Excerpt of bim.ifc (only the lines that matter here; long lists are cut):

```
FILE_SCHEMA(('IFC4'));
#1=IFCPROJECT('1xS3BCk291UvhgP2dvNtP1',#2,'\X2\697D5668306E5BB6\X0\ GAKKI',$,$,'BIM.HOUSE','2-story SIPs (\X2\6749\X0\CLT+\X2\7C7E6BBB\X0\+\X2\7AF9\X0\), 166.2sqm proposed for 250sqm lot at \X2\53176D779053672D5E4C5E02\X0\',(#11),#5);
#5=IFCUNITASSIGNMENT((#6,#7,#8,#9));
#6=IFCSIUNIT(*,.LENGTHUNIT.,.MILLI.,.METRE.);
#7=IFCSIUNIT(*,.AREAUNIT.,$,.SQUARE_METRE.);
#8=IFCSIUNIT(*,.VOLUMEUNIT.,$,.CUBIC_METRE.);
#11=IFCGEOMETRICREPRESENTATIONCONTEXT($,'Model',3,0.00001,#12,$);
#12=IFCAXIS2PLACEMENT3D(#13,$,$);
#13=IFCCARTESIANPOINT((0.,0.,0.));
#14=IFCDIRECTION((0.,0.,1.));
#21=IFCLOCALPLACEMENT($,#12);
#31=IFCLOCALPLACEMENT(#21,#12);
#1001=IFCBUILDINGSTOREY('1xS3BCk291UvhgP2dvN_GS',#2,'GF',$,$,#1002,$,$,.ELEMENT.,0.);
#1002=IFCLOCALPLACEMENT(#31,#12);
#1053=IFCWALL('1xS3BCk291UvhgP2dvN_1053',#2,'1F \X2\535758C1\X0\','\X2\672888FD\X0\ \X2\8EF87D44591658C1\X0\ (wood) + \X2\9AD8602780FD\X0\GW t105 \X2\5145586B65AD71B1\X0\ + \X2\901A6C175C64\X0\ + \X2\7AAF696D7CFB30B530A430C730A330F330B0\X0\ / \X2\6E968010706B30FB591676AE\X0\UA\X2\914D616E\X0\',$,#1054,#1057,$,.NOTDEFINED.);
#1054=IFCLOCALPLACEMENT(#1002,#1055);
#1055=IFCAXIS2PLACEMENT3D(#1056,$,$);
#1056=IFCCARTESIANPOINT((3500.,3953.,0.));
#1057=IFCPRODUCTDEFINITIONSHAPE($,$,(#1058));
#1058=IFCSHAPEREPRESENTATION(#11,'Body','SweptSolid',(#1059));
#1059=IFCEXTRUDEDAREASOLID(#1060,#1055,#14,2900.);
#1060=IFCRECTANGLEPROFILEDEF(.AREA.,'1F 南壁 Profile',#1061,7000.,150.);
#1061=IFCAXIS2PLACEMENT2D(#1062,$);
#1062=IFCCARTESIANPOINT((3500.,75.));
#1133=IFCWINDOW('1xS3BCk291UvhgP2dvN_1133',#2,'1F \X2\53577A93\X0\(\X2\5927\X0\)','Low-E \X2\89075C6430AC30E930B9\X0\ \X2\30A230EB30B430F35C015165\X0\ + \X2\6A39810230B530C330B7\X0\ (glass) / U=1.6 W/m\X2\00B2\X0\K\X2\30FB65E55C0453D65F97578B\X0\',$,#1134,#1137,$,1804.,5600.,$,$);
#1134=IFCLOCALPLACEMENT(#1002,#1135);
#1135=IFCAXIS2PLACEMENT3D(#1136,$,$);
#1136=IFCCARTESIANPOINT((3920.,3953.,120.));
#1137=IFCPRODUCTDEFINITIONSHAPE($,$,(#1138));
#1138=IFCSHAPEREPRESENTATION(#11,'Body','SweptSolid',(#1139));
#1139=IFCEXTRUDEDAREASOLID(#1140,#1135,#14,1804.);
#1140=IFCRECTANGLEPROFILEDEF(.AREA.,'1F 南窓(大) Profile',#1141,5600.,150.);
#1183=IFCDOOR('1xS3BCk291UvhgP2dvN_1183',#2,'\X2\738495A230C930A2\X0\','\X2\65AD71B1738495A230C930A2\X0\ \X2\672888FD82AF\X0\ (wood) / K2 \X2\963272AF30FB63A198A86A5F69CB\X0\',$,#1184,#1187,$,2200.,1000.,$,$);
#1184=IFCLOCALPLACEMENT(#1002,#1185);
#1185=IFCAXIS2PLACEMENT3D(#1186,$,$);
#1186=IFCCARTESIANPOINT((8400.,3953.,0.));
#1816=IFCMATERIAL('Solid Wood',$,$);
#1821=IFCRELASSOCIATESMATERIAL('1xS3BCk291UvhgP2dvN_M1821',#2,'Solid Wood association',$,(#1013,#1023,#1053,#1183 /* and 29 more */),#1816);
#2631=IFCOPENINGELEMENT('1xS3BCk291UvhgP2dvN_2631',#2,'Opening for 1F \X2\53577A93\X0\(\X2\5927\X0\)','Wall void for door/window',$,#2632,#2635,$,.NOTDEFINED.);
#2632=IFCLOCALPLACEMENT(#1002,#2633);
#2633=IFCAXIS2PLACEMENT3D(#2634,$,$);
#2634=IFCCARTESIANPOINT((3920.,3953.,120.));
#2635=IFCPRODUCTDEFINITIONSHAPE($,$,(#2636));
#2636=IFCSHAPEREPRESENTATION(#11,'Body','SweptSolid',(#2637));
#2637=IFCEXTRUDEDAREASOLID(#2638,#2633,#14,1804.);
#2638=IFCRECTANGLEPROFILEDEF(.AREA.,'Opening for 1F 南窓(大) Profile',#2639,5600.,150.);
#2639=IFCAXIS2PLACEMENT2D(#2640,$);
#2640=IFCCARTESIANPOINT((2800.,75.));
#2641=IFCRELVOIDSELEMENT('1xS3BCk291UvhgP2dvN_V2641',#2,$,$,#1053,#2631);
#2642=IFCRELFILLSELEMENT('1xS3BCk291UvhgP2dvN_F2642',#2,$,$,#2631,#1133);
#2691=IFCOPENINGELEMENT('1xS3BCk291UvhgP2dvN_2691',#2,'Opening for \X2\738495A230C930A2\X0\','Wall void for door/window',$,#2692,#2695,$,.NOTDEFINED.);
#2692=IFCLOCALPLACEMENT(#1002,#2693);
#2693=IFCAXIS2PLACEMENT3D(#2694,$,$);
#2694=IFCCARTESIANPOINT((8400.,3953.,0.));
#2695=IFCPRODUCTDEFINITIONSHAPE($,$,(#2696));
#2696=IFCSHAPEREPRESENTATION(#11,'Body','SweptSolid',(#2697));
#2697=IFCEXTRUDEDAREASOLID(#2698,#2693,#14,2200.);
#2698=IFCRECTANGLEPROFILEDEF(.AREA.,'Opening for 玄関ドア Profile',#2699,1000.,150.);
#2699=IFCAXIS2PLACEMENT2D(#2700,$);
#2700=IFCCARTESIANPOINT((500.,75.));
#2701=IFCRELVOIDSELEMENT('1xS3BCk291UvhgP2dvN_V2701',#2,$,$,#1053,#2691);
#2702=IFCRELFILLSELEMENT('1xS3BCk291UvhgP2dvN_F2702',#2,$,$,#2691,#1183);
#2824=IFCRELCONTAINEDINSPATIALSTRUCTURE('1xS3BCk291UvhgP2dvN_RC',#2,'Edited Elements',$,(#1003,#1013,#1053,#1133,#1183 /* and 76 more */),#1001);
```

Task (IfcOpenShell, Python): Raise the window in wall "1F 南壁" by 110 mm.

```python
import numpy as np
import ifcopenshell
import ifcopenshell.api.geometry
import ifcopenshell.util.placement
import ifcopenshell.util.unit

model = ifcopenshell.open("bim.ifc")
unit_scale = ifcopenshell.util.unit.calculate_unit_scale(model)

window = model.by_id(1133)
opening = window.FillsVoids[0].RelatingOpeningElement
dz = 0.11 / unit_scale

shift = np.array([0.0, 0.0, dz])
# The window is not placed relative to its opening, so move both.
for product in (opening, window):
    matrix = ifcopenshell.util.placement.get_local_placement(product.ObjectPlacement)
    matrix[:3, 3] += shift
    ifcopenshell.api.geometry.edit_object_placement(model, product=product, matrix=matrix, is_si=False)

print(f"moved by {dz * unit_scale:+.3f} m")

model.write("bim_edited.ifc")
```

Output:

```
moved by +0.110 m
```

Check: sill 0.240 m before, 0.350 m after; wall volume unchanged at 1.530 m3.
